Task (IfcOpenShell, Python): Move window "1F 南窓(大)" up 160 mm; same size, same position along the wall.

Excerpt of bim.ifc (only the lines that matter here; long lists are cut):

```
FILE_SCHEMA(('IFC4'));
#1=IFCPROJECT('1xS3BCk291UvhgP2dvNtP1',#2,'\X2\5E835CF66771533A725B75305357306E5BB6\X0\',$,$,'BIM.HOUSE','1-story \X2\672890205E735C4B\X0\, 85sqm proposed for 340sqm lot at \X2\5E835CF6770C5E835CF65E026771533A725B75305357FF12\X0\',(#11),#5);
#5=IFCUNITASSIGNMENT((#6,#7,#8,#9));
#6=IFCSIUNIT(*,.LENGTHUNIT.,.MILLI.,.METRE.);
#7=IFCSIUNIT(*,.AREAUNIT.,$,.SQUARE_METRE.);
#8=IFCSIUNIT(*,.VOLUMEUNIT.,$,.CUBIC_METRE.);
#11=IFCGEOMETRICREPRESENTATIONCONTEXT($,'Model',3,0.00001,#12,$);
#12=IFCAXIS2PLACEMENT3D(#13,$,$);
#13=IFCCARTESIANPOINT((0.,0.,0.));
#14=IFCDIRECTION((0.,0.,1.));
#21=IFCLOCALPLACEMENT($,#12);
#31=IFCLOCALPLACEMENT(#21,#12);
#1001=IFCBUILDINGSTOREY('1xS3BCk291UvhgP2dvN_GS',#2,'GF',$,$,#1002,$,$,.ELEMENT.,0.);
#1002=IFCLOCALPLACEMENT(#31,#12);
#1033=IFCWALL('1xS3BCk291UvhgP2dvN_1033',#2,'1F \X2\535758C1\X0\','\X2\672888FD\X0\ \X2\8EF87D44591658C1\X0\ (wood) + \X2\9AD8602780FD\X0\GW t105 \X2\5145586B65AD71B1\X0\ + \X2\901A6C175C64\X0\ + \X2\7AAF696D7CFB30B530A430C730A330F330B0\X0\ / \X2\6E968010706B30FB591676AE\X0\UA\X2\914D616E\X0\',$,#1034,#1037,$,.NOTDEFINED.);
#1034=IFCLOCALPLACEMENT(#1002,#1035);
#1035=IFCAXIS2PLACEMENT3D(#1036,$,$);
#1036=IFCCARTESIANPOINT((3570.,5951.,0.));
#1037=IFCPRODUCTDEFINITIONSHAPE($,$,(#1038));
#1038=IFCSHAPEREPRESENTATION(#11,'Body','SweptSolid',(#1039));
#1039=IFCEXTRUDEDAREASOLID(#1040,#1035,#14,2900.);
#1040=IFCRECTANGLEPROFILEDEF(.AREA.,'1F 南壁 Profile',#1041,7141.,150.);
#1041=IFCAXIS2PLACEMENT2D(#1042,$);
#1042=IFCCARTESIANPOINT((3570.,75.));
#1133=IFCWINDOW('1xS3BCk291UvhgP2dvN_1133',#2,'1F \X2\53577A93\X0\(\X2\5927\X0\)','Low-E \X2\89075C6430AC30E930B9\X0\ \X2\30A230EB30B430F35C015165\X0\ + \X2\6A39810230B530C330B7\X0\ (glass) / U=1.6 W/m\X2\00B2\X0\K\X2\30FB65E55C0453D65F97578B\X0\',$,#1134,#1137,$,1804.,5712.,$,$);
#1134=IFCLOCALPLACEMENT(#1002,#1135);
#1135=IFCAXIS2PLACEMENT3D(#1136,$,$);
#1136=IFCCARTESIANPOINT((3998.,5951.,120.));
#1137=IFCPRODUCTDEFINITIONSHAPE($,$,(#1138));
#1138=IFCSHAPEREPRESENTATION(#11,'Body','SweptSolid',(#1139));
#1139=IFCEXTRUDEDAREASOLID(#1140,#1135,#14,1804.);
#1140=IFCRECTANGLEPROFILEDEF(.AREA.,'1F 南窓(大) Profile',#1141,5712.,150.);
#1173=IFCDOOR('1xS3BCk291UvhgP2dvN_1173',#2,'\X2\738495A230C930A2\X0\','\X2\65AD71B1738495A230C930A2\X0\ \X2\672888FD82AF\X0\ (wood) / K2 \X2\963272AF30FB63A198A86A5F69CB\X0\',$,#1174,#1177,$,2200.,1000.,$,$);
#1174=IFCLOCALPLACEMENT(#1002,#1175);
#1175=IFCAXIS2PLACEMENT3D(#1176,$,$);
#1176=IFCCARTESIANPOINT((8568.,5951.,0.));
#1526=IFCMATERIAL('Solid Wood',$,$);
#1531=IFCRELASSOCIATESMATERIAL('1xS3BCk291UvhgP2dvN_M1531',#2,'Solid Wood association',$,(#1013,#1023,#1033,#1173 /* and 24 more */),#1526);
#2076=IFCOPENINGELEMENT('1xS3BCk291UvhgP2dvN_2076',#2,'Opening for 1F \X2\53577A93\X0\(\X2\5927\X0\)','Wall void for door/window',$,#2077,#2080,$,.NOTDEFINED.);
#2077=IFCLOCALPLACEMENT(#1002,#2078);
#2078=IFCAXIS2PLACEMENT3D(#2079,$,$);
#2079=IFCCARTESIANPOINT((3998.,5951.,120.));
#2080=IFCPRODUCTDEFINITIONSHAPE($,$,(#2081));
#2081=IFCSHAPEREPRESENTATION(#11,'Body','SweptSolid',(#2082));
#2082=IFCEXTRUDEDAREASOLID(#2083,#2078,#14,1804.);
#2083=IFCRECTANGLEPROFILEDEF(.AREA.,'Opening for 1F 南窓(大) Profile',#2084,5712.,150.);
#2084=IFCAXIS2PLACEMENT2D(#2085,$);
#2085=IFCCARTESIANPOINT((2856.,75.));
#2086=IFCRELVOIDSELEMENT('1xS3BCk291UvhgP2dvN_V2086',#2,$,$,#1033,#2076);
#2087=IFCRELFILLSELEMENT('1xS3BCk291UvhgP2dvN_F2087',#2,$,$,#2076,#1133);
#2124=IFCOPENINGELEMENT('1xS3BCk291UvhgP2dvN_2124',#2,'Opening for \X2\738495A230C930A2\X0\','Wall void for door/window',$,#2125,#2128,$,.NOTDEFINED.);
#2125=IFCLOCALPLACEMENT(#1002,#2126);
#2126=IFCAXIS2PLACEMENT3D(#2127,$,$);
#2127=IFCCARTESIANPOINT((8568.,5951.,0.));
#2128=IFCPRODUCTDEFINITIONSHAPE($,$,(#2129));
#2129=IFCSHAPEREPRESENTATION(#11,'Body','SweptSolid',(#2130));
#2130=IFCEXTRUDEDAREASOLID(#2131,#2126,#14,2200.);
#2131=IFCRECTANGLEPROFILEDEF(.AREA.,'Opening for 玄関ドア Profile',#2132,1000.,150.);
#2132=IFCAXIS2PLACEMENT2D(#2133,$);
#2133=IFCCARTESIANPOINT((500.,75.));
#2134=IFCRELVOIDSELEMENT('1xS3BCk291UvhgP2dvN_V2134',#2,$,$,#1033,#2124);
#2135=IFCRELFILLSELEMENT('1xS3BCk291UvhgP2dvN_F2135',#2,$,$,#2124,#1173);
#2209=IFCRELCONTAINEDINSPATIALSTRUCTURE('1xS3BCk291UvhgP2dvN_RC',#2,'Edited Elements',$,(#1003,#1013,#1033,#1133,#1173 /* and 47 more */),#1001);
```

```python
import numpy as np
import ifcopenshell
import ifcopenshell.api.geometry
import ifcopenshell.util.placement
import ifcopenshell.util.unit

model = ifcopenshell.open("bim.ifc")
unit_scale = ifcopenshell.util.unit.calculate_unit_scale(model)

window = model.by_guid("1xS3BCk291UvhgP2dvN_1133")
opening = window.FillsVoids[0].RelatingOpeningElement
dz = 0.16 / unit_scale

shift = np.array([0.0, 0.0, dz])
# The window is not placed relative to its opening, so move both.
for product in (opening, window):
    matrix = ifcopenshell.util.placement.get_local_placement(product.ObjectPlacement)
    matrix[:3, 3] += shift
    ifcopenshell.api.geometry.edit_object_placement(model, product=product, matrix=matrix, is_si=False)

print(f"moved by {dz * unit_scale:+.3f} m")

model.write("bim_v2.ifc")
```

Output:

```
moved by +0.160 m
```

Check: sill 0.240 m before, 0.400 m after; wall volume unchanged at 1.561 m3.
